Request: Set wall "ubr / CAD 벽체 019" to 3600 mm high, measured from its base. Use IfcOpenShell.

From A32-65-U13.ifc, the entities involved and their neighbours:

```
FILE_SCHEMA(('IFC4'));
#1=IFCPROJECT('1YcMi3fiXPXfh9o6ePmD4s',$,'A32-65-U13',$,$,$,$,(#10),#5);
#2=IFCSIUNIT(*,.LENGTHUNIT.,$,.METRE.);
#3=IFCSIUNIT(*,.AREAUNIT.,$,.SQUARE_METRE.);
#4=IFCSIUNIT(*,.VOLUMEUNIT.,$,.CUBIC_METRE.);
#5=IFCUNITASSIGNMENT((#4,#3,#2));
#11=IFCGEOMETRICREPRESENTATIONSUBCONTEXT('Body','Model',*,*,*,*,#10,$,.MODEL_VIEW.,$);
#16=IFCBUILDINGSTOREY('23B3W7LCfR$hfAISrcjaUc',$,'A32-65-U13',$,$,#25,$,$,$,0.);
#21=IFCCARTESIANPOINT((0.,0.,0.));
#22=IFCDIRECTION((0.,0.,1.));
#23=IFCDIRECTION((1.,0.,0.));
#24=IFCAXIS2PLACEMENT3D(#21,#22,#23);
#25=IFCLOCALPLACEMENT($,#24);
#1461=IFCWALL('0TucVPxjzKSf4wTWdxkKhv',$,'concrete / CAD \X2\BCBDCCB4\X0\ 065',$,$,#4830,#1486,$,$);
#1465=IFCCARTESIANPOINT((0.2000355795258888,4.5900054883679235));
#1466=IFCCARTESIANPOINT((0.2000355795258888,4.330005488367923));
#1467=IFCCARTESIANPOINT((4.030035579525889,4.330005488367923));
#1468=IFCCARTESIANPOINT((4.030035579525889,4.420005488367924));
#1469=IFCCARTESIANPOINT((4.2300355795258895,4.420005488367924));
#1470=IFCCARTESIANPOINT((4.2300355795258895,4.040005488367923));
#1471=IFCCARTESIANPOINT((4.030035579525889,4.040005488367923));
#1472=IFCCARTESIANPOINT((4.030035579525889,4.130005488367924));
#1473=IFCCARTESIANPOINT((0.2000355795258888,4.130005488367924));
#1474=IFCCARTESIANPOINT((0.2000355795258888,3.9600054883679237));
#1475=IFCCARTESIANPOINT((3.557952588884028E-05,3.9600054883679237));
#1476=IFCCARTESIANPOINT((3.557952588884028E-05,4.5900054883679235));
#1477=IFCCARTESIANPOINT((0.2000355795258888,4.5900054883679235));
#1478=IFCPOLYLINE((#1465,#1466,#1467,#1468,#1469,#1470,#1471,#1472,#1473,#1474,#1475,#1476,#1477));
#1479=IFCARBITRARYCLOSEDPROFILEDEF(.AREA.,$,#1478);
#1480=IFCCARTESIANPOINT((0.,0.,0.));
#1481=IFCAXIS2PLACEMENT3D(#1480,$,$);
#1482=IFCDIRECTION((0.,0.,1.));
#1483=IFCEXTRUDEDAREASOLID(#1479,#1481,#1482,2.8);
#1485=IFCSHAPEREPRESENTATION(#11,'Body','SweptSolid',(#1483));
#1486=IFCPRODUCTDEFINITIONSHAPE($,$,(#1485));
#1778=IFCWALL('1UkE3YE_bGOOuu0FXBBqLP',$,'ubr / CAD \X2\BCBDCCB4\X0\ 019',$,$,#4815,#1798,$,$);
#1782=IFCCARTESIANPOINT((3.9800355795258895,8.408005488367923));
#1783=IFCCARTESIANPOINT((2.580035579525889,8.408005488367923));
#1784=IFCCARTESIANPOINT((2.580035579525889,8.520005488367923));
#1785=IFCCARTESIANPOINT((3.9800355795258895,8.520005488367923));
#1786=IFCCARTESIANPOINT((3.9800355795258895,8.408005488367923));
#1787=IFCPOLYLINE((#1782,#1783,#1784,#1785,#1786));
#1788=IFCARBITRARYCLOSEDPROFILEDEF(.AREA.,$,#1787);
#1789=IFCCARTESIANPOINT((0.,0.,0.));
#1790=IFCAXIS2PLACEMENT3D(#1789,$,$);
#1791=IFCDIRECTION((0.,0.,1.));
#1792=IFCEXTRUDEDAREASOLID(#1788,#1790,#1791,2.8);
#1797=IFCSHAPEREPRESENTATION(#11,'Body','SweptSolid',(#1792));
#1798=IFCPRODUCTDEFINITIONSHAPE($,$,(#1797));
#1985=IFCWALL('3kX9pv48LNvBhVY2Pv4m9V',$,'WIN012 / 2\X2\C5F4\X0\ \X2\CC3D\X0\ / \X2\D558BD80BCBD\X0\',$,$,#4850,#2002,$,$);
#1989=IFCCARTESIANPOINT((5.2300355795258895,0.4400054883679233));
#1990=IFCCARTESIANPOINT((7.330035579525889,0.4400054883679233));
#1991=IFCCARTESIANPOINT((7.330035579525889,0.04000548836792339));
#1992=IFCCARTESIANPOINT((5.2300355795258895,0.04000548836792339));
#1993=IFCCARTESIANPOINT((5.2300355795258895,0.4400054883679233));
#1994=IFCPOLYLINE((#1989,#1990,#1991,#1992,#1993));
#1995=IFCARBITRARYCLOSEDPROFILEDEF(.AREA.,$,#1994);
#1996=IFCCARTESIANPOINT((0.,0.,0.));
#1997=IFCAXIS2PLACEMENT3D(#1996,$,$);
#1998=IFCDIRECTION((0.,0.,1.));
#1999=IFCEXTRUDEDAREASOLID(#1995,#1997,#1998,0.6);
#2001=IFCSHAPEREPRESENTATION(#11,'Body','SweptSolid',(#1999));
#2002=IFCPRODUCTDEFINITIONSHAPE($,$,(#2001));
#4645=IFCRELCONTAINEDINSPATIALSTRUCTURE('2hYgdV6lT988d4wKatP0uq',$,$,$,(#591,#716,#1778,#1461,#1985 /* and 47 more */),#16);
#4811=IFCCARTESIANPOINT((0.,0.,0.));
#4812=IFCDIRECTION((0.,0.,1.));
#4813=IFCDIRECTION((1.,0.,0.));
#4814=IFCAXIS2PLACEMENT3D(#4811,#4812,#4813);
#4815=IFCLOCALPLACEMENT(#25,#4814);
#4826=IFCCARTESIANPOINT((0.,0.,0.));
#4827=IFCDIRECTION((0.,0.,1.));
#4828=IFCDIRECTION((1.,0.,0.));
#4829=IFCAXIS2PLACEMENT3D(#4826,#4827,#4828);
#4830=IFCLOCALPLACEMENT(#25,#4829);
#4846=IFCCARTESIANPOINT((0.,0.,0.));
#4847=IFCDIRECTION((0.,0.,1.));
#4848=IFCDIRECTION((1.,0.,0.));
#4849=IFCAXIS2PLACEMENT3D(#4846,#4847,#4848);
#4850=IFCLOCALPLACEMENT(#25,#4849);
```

```python
import ifcopenshell
import ifcopenshell.geom
import ifcopenshell.util.representation
import ifcopenshell.util.shape
import ifcopenshell.util.unit

model = ifcopenshell.open("A32-65-U13.ifc")
unit_scale = ifcopenshell.util.unit.calculate_unit_scale(model)
settings = ifcopenshell.geom.settings()


def volume(element):
    """Net volume in cubic metres, openings subtracted."""
    shape = ifcopenshell.geom.create_shape(settings, element)
    return ifcopenshell.util.shape.get_volume(shape.geometry)


wall = model.by_id(1778)
before = volume(wall)

body = ifcopenshell.util.representation.get_representation(wall, "Model", "Body")
solid = body.Items[0]
old_height = solid.Depth
solid.Depth = 3.6 / unit_scale
after = volume(wall)

print(f"height {old_height:g} -> {solid.Depth:g}, volume {before:.3f} -> {after:.3f} m3")

model.write("A32-65-U13_v2.ifc")
```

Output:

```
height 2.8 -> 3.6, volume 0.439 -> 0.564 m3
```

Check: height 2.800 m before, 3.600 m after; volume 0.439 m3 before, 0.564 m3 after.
